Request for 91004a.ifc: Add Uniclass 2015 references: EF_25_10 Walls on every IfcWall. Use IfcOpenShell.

First a look at what the model holds.

```python
import ifcopenshell

model = ifcopenshell.open("91004a.ifc")
print(model.schema)
print("classifications:", [c.Name for c in model.by_type("IfcClassification")])
for ifc_class in ("IfcDoor", "IfcRoof", "IfcStair", "IfcWall", "IfcWindow"):
    print(ifc_class, len(model.by_type(ifc_class)))
```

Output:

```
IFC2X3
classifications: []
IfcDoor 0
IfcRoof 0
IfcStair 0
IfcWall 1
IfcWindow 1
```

```python
import ifcopenshell
import ifcopenshell.api.classification

model = ifcopenshell.open("91004a.ifc")

# IFC2X3 requires Source and Edition and has no link from the project to the system.
system = model.create_entity("IfcClassification", Source="NBS", Edition="2015", Name="Uniclass 2015")

codes = {
    "IfcWall": ("EF_25_10", "Walls"),
}
for ifc_class, (code, name) in codes.items():
    products = model.by_type(ifc_class)
    ifcopenshell.api.classification.add_reference(
        model, products=products, classification=system, identification=code, name=name
    )
    print(code, len(products))

model.write("91004a-out.ifc")
```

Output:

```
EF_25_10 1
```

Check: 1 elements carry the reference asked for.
